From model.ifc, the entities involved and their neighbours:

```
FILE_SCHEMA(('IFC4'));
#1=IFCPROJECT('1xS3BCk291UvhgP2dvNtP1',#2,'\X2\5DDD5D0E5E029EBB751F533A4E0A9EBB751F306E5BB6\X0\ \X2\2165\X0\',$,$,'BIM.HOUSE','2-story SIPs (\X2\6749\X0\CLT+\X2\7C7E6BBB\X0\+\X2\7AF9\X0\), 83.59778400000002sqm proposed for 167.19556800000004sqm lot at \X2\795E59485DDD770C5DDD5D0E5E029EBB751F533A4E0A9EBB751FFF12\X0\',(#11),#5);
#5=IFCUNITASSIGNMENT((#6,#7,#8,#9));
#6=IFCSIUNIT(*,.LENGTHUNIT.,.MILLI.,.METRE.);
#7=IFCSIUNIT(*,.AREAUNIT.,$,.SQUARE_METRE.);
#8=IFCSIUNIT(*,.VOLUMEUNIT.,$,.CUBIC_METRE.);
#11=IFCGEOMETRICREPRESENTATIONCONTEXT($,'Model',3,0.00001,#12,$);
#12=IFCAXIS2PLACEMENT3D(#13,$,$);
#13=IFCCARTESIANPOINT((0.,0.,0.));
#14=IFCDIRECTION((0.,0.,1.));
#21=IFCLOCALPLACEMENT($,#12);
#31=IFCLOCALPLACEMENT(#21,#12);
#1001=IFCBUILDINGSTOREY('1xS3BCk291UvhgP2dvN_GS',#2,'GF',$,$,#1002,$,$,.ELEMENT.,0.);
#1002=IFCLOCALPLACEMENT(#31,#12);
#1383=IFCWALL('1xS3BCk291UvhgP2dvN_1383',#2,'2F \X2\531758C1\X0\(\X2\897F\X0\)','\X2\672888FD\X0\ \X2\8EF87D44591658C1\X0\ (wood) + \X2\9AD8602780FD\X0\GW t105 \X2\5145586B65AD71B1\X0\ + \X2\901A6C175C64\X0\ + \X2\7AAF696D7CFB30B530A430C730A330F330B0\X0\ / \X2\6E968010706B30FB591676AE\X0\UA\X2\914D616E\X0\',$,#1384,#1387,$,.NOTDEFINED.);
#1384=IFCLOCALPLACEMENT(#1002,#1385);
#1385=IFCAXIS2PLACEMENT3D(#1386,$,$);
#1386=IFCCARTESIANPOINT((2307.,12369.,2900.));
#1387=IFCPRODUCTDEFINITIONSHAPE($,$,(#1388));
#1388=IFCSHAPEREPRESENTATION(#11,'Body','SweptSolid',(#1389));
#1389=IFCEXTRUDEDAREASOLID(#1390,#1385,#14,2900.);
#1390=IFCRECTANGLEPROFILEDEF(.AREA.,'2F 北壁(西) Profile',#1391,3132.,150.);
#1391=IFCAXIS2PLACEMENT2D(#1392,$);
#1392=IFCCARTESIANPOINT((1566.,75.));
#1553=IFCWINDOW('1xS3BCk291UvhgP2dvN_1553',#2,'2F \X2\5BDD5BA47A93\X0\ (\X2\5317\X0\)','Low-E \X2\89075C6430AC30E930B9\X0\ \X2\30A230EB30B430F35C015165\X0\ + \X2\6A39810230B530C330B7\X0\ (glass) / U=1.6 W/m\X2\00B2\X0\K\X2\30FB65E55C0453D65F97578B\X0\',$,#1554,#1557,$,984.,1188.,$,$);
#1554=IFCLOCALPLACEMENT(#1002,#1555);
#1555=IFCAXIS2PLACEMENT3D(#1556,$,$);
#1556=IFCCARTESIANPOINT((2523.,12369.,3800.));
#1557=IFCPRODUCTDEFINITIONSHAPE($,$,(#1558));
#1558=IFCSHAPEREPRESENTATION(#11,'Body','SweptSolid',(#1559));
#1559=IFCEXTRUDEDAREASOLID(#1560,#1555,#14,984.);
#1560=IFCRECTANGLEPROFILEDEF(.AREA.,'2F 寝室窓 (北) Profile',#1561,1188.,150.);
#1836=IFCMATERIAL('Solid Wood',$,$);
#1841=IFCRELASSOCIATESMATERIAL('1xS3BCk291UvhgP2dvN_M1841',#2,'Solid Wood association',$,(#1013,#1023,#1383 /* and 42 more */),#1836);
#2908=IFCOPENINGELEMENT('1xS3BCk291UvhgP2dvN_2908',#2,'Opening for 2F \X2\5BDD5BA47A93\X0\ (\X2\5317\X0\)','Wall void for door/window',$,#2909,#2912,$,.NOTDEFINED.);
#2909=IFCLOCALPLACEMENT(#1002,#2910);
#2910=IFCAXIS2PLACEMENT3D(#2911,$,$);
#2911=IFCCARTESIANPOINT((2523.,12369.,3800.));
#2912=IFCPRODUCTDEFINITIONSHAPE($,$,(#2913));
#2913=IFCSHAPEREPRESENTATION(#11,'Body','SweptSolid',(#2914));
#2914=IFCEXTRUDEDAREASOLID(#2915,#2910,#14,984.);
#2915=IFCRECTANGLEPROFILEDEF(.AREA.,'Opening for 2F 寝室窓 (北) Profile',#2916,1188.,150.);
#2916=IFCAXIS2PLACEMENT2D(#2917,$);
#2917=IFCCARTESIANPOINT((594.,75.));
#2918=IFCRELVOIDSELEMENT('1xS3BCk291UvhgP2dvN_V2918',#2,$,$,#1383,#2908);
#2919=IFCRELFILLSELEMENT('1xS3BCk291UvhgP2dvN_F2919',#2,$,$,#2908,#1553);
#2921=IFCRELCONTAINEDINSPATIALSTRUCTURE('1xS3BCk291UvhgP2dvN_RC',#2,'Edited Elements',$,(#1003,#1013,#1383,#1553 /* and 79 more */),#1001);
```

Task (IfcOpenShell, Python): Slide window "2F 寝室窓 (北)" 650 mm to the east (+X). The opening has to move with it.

```python
import ifcopenshell
import ifcopenshell.api.geometry
import ifcopenshell.util.placement
import ifcopenshell.util.unit

model = ifcopenshell.open("model.ifc")
unit_scale = ifcopenshell.util.unit.calculate_unit_scale(model)

window = model.by_guid("1xS3BCk291UvhgP2dvN_1553")
opening = window.FillsVoids[0].RelatingOpeningElement
wall = opening.VoidsElements[0].RelatingBuildingElement

wall_matrix = ifcopenshell.util.placement.get_local_placement(wall.ObjectPlacement)
shift = wall_matrix[:3, 0] * 0.65 / unit_scale
before = ifcopenshell.util.placement.get_local_placement(window.ObjectPlacement)[:3, 3].copy()

# The window is not placed relative to its opening, so move both.
for product in (opening, window):
    matrix = ifcopenshell.util.placement.get_local_placement(product.ObjectPlacement)
    matrix[:3, 3] += shift
    ifcopenshell.api.geometry.edit_object_placement(model, product=product, matrix=matrix, is_si=False)

after = ifcopenshell.util.placement.get_local_placement(window.ObjectPlacement)[:3, 3]
print("window moved by", (after - before).round(3) + 0.0)

model.write("model_edited.ifc")
```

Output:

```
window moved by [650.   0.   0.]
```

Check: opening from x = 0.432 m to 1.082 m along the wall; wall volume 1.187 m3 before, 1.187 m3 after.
